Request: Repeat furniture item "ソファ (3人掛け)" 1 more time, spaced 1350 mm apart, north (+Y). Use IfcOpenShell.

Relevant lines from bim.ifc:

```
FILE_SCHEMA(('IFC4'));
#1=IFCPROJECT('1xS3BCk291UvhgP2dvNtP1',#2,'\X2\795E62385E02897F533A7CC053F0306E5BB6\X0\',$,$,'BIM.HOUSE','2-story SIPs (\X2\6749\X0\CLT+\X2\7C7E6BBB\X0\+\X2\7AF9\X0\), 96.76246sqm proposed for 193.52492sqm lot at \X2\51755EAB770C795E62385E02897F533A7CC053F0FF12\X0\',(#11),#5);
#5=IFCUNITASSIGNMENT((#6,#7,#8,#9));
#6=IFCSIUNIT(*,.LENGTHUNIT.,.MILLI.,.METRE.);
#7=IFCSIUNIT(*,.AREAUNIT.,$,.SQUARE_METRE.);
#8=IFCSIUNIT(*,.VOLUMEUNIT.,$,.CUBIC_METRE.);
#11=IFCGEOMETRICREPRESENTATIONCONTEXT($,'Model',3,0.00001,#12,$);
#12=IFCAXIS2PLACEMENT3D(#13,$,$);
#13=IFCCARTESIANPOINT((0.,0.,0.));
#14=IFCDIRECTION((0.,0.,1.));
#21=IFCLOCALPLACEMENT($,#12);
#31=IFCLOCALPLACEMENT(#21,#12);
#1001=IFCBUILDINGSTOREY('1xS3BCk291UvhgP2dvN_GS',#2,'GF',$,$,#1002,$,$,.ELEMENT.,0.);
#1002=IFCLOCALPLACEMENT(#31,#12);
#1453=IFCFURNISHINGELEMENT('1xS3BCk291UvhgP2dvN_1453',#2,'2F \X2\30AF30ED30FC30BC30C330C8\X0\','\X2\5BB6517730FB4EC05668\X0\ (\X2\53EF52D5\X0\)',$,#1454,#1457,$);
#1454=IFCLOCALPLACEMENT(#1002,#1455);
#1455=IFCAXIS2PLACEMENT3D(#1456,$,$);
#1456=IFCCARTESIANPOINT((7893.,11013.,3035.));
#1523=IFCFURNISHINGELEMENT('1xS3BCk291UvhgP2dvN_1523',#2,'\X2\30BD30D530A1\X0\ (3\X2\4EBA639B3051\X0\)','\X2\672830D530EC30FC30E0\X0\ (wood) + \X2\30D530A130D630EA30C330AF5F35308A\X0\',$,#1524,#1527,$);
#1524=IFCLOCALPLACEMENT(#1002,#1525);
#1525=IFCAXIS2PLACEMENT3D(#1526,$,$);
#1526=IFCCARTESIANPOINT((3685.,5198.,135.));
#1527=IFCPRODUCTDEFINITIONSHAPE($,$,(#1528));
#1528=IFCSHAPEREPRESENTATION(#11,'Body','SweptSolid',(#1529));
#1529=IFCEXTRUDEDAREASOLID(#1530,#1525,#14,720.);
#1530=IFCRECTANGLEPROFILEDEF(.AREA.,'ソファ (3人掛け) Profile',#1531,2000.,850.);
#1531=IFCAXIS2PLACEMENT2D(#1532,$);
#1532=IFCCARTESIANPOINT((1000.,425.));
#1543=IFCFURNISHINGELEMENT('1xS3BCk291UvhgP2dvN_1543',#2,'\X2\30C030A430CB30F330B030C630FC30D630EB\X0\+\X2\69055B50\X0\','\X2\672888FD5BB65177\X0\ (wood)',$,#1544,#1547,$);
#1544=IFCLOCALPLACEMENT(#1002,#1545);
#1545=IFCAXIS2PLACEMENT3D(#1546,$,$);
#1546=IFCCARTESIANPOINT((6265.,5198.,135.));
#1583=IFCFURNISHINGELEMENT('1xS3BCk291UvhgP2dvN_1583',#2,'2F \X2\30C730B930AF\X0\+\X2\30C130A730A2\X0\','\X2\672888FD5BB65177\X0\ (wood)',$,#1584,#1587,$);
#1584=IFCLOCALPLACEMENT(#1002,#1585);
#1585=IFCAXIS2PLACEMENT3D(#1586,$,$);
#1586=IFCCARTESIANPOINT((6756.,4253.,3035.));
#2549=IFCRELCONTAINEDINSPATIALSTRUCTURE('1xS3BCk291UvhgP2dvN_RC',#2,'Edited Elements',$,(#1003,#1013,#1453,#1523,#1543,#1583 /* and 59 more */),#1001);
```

```python
import numpy as np
import ifcopenshell
import ifcopenshell.api.geometry
import ifcopenshell.api.root
import ifcopenshell.util.element
import ifcopenshell.util.placement
import ifcopenshell.util.unit

model = ifcopenshell.open("bim.ifc")
unit_scale = ifcopenshell.util.unit.calculate_unit_scale(model)


def reuse_history(source, copy):
    """copy_class also copies each property set's owner history, people and application; keep the originals."""
    for rel in copy.IsDefinedBy:
        if rel.is_a("IfcRelDefinesByProperties") and (history := rel.RelatingPropertyDefinition.OwnerHistory):
            rel.RelatingPropertyDefinition.OwnerHistory = source.OwnerHistory
            ifcopenshell.util.element.remove_deep2(model, history)


source = model.by_guid("1xS3BCk291UvhgP2dvN_1523")
base = ifcopenshell.util.placement.get_local_placement(source.ObjectPlacement)
step = np.array([0.0, 1.0, 0.0]) * 1.35 / unit_scale

for i in range(1, 2):
    copy = ifcopenshell.api.root.copy_class(model, product=source)
    copy.Representation = ifcopenshell.util.element.copy_deep(
        model, source.Representation, exclude=["IfcGeometricRepresentationContext", "IfcRepresentationMap"]
    )
    reuse_history(source, copy)
    matrix = base.copy()
    matrix[:3, 3] += i * step
    print("added at", matrix[:3, 3].round(3) + 0.0)
    ifcopenshell.api.geometry.edit_object_placement(model, product=copy, matrix=matrix, is_si=False)

model.write("bim-out.ifc")
```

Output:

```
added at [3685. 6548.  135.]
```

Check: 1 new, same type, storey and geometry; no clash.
